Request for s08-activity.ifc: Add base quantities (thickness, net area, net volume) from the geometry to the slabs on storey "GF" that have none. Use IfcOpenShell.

First a look at what the model holds.

```python
import ifcopenshell
import ifcopenshell.util.element
import ifcopenshell.util.unit

model = ifcopenshell.open("s08-activity.ifc")
print(model.schema)
for unit_type in ("LENGTHUNIT", "AREAUNIT", "VOLUMEUNIT"):
    print(unit_type, ifcopenshell.util.unit.calculate_unit_scale(model, unit_type))
storey = next(s for s in model.by_type("IfcBuildingStorey") if s.Name == "GF")
slabs = [e for e in ifcopenshell.util.element.get_decomposition(storey) if e.is_a("IfcSlab")]
for e in sorted(slabs, key=lambda e: e.id()):
    print(e.id(), e.is_a(), e.Name, list(ifcopenshell.util.element.get_psets(e, qtos_only=True)), sep=" | ")
```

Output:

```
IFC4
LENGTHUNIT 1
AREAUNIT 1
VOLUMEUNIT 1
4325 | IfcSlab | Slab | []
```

```python
import ifcopenshell
import ifcopenshell.api.pset
import ifcopenshell.geom
import ifcopenshell.util.element
import ifcopenshell.util.shape
import ifcopenshell.util.unit

model = ifcopenshell.open("s08-activity.ifc")
unit_scale = ifcopenshell.util.unit.calculate_unit_scale(model)
area_scale = ifcopenshell.util.unit.calculate_unit_scale(model, "AREAUNIT")
volume_scale = ifcopenshell.util.unit.calculate_unit_scale(model, "VOLUMEUNIT")
settings = ifcopenshell.geom.settings()

storey = next(s for s in model.by_type("IfcBuildingStorey") if s.Name == "GF")
slabs = [e for e in ifcopenshell.util.element.get_decomposition(storey) if e.is_a("IfcSlab")]

for e in sorted(slabs, key=lambda e: e.id()):
    if ifcopenshell.util.element.get_psets(e, qtos_only=True, should_inherit=False):
        continue
    # Geometry comes back in metres, in the element's own axes.
    shape = ifcopenshell.geom.create_shape(settings, e)
    values = {
        "Width": ifcopenshell.util.shape.get_z(shape.geometry) / unit_scale,
        "NetArea": ifcopenshell.util.shape.get_footprint_area(shape.geometry) / area_scale,
        "NetVolume": ifcopenshell.util.shape.get_volume(shape.geometry) / volume_scale,
    }
    qto = ifcopenshell.api.pset.add_qto(model, product=e, name="Qto_SlabBaseQuantities")
    ifcopenshell.api.pset.edit_qto(model, qto=qto, properties=values)
    print(e.id(), {k: round(v, 3) for k, v in values.items()})

model.write("s08-activity_v2.ifc")
```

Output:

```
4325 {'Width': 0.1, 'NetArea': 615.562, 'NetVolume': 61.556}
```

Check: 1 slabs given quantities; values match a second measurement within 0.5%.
